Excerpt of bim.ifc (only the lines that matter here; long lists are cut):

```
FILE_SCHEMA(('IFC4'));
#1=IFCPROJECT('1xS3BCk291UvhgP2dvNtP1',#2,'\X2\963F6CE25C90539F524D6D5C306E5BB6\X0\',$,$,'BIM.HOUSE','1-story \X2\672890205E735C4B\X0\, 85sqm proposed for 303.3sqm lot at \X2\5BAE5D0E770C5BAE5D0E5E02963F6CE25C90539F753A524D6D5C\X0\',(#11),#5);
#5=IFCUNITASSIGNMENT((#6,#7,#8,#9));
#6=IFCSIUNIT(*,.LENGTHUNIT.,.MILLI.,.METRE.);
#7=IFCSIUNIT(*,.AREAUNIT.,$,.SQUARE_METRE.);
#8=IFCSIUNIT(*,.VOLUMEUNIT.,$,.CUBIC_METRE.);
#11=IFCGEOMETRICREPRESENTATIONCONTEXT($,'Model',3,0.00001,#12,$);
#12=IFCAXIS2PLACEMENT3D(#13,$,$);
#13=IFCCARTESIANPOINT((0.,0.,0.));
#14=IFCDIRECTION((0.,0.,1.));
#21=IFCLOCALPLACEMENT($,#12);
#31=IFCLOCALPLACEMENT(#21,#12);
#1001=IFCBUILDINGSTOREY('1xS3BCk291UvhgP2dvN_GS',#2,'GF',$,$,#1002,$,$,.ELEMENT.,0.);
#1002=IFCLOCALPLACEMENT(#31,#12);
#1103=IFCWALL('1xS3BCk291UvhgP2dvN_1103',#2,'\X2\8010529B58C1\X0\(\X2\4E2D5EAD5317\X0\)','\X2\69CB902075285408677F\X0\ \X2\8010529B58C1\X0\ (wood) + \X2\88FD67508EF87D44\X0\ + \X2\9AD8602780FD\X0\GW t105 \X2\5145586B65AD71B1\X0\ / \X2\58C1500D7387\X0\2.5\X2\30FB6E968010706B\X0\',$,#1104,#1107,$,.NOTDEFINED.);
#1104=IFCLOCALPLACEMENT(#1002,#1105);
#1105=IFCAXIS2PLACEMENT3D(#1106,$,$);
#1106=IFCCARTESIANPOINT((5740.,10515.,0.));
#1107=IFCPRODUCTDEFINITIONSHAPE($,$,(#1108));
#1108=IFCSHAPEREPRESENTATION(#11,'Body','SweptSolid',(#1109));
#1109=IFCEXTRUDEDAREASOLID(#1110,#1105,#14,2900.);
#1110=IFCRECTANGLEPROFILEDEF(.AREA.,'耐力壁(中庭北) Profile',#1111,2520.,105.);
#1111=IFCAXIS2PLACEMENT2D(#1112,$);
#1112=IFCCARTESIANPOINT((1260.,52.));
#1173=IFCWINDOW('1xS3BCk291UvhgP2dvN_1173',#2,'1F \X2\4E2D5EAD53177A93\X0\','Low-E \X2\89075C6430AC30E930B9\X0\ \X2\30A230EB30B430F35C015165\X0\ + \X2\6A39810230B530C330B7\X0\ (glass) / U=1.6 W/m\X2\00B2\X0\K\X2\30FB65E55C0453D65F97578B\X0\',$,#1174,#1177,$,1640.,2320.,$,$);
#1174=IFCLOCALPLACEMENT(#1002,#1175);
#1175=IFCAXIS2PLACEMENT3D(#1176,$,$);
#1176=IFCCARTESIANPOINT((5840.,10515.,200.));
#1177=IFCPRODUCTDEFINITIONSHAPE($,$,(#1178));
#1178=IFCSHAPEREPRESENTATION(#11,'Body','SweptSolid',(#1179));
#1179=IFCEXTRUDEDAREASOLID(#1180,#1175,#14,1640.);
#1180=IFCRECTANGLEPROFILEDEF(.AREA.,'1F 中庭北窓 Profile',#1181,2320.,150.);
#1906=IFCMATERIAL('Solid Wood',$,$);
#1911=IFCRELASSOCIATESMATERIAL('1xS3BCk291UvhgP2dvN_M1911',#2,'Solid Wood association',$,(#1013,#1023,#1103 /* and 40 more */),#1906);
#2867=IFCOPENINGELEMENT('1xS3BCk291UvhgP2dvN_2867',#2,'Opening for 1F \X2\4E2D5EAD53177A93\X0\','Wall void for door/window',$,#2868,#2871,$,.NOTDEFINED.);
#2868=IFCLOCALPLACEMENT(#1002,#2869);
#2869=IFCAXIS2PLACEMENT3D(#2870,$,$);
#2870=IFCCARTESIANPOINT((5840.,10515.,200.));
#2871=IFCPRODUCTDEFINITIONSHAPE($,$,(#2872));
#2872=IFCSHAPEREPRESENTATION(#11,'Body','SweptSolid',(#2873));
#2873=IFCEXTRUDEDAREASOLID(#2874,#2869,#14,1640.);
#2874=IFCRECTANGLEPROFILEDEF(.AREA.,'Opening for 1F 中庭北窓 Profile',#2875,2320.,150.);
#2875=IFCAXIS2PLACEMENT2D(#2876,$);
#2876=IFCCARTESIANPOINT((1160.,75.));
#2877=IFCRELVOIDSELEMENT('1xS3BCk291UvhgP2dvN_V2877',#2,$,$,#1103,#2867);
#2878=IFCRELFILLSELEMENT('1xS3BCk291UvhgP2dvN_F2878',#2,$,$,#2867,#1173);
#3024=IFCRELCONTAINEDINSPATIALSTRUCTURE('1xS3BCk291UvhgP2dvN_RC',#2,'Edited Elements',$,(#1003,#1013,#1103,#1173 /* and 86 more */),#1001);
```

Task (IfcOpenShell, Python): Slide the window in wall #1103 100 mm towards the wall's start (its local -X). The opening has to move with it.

```python
import ifcopenshell
import ifcopenshell.api.geometry
import ifcopenshell.util.placement

model = ifcopenshell.open("bim.ifc")

window = model.by_id(1173)
opening = window.FillsVoids[0].RelatingOpeningElement
wall = opening.VoidsElements[0].RelatingBuildingElement

wall_matrix = ifcopenshell.util.placement.get_local_placement(wall.ObjectPlacement)
shift = wall_matrix[:3, 0] * -100.0
before = ifcopenshell.util.placement.get_local_placement(window.ObjectPlacement)[:3, 3].copy()

# The window is not placed relative to its opening, so move both.
for product in (opening, window):
    matrix = ifcopenshell.util.placement.get_local_placement(product.ObjectPlacement)
    matrix[:3, 3] += shift
    ifcopenshell.api.geometry.edit_object_placement(model, product=product, matrix=matrix, is_si=False)

after = ifcopenshell.util.placement.get_local_placement(window.ObjectPlacement)[:3, 3]
print("window moved by", (after - before).round(3) + 0.0)

model.write("bim_updated.ifc")
```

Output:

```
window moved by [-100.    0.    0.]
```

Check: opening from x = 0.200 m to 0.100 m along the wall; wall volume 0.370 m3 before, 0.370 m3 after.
